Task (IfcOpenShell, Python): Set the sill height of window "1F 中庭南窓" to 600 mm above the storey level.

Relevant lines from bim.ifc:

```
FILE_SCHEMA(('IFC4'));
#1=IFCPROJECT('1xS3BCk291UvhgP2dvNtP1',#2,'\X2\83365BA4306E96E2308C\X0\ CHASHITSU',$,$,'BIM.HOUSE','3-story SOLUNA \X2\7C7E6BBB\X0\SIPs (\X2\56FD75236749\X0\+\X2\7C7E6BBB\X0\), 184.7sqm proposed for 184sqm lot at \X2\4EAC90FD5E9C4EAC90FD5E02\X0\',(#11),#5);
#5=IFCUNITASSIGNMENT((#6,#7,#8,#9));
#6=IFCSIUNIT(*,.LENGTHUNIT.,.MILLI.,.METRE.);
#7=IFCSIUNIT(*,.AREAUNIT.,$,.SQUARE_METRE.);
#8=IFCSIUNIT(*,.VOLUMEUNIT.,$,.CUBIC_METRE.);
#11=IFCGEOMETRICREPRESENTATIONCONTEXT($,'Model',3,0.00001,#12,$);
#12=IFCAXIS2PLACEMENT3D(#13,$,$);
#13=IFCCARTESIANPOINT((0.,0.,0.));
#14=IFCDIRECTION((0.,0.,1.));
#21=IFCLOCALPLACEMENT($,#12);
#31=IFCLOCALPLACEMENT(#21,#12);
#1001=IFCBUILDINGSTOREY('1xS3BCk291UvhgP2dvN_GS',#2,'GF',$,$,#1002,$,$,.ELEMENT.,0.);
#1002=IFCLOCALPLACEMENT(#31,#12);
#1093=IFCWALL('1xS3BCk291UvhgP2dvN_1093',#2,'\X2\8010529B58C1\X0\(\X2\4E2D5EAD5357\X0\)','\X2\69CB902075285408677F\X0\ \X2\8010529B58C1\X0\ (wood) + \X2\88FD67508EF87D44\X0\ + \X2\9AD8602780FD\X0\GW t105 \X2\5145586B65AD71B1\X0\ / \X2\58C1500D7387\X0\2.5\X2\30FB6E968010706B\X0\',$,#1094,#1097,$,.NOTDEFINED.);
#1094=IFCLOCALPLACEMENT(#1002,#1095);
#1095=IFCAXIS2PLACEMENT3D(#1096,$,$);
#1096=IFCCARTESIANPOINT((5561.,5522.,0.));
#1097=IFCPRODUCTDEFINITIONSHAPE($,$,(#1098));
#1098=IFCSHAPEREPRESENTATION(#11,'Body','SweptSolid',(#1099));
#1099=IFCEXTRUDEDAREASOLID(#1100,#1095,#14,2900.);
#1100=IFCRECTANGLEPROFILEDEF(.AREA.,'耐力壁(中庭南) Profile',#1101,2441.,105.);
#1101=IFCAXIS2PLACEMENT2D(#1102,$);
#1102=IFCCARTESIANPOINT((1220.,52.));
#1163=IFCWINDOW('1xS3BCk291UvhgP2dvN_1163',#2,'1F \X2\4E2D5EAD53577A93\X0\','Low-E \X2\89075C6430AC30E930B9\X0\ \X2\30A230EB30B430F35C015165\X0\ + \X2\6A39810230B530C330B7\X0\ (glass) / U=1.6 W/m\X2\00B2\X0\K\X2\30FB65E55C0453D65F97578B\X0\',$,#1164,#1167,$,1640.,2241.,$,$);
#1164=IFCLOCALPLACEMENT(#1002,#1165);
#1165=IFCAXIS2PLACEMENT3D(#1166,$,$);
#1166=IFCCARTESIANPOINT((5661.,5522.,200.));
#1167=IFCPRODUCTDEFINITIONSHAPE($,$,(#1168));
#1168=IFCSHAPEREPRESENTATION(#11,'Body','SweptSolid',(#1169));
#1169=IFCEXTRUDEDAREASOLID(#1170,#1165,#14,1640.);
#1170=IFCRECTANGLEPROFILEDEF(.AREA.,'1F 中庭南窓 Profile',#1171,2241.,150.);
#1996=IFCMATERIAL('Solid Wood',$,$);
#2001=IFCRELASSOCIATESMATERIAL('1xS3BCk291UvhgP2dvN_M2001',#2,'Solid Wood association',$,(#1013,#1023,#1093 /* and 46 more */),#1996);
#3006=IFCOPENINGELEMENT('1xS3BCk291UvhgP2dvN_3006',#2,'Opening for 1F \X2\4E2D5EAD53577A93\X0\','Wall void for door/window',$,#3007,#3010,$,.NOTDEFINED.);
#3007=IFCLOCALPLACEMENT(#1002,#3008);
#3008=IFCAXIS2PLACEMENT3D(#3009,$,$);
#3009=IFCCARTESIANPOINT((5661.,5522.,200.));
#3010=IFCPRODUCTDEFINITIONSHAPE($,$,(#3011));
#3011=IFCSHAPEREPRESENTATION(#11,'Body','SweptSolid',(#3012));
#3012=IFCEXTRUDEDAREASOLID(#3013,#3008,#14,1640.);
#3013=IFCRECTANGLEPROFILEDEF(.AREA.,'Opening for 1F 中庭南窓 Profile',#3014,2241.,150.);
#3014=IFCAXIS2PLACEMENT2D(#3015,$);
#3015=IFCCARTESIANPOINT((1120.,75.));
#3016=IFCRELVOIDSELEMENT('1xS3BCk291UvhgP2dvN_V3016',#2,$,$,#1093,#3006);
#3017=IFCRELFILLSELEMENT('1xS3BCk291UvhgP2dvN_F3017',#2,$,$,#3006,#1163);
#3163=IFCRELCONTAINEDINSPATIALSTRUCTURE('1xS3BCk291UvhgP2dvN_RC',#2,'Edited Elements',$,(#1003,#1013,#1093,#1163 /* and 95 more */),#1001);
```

```python
import numpy as np
import ifcopenshell
import ifcopenshell.api.geometry
import ifcopenshell.geom
import ifcopenshell.util.element
import ifcopenshell.util.placement
import ifcopenshell.util.shape
import ifcopenshell.util.unit

model = ifcopenshell.open("bim.ifc")
unit_scale = ifcopenshell.util.unit.calculate_unit_scale(model)

window = model.by_id(1163)
opening = window.FillsVoids[0].RelatingOpeningElement
storey = ifcopenshell.util.element.get_container(window, ifc_class="IfcBuildingStorey")
level = ifcopenshell.util.placement.get_local_placement(storey.ObjectPlacement)[2, 3]

# The opening's origin need not be at the sill, so measure its lowest point.
shape = ifcopenshell.geom.create_shape(ifcopenshell.geom.settings(), opening)
bottom = ifcopenshell.util.shape.get_shape_bottom_elevation(shape, shape.geometry) / unit_scale
dz = level + 0.6 / unit_scale - bottom

shift = np.array([0.0, 0.0, dz])
# The window is not placed relative to its opening, so move both.
for product in (opening, window):
    matrix = ifcopenshell.util.placement.get_local_placement(product.ObjectPlacement)
    matrix[:3, 3] += shift
    ifcopenshell.api.geometry.edit_object_placement(model, product=product, matrix=matrix, is_si=False)

print(f"moved by {dz * unit_scale:+.3f} m")

model.write("bim-out.ifc")
```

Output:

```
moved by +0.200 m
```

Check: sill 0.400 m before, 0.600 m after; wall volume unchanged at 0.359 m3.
